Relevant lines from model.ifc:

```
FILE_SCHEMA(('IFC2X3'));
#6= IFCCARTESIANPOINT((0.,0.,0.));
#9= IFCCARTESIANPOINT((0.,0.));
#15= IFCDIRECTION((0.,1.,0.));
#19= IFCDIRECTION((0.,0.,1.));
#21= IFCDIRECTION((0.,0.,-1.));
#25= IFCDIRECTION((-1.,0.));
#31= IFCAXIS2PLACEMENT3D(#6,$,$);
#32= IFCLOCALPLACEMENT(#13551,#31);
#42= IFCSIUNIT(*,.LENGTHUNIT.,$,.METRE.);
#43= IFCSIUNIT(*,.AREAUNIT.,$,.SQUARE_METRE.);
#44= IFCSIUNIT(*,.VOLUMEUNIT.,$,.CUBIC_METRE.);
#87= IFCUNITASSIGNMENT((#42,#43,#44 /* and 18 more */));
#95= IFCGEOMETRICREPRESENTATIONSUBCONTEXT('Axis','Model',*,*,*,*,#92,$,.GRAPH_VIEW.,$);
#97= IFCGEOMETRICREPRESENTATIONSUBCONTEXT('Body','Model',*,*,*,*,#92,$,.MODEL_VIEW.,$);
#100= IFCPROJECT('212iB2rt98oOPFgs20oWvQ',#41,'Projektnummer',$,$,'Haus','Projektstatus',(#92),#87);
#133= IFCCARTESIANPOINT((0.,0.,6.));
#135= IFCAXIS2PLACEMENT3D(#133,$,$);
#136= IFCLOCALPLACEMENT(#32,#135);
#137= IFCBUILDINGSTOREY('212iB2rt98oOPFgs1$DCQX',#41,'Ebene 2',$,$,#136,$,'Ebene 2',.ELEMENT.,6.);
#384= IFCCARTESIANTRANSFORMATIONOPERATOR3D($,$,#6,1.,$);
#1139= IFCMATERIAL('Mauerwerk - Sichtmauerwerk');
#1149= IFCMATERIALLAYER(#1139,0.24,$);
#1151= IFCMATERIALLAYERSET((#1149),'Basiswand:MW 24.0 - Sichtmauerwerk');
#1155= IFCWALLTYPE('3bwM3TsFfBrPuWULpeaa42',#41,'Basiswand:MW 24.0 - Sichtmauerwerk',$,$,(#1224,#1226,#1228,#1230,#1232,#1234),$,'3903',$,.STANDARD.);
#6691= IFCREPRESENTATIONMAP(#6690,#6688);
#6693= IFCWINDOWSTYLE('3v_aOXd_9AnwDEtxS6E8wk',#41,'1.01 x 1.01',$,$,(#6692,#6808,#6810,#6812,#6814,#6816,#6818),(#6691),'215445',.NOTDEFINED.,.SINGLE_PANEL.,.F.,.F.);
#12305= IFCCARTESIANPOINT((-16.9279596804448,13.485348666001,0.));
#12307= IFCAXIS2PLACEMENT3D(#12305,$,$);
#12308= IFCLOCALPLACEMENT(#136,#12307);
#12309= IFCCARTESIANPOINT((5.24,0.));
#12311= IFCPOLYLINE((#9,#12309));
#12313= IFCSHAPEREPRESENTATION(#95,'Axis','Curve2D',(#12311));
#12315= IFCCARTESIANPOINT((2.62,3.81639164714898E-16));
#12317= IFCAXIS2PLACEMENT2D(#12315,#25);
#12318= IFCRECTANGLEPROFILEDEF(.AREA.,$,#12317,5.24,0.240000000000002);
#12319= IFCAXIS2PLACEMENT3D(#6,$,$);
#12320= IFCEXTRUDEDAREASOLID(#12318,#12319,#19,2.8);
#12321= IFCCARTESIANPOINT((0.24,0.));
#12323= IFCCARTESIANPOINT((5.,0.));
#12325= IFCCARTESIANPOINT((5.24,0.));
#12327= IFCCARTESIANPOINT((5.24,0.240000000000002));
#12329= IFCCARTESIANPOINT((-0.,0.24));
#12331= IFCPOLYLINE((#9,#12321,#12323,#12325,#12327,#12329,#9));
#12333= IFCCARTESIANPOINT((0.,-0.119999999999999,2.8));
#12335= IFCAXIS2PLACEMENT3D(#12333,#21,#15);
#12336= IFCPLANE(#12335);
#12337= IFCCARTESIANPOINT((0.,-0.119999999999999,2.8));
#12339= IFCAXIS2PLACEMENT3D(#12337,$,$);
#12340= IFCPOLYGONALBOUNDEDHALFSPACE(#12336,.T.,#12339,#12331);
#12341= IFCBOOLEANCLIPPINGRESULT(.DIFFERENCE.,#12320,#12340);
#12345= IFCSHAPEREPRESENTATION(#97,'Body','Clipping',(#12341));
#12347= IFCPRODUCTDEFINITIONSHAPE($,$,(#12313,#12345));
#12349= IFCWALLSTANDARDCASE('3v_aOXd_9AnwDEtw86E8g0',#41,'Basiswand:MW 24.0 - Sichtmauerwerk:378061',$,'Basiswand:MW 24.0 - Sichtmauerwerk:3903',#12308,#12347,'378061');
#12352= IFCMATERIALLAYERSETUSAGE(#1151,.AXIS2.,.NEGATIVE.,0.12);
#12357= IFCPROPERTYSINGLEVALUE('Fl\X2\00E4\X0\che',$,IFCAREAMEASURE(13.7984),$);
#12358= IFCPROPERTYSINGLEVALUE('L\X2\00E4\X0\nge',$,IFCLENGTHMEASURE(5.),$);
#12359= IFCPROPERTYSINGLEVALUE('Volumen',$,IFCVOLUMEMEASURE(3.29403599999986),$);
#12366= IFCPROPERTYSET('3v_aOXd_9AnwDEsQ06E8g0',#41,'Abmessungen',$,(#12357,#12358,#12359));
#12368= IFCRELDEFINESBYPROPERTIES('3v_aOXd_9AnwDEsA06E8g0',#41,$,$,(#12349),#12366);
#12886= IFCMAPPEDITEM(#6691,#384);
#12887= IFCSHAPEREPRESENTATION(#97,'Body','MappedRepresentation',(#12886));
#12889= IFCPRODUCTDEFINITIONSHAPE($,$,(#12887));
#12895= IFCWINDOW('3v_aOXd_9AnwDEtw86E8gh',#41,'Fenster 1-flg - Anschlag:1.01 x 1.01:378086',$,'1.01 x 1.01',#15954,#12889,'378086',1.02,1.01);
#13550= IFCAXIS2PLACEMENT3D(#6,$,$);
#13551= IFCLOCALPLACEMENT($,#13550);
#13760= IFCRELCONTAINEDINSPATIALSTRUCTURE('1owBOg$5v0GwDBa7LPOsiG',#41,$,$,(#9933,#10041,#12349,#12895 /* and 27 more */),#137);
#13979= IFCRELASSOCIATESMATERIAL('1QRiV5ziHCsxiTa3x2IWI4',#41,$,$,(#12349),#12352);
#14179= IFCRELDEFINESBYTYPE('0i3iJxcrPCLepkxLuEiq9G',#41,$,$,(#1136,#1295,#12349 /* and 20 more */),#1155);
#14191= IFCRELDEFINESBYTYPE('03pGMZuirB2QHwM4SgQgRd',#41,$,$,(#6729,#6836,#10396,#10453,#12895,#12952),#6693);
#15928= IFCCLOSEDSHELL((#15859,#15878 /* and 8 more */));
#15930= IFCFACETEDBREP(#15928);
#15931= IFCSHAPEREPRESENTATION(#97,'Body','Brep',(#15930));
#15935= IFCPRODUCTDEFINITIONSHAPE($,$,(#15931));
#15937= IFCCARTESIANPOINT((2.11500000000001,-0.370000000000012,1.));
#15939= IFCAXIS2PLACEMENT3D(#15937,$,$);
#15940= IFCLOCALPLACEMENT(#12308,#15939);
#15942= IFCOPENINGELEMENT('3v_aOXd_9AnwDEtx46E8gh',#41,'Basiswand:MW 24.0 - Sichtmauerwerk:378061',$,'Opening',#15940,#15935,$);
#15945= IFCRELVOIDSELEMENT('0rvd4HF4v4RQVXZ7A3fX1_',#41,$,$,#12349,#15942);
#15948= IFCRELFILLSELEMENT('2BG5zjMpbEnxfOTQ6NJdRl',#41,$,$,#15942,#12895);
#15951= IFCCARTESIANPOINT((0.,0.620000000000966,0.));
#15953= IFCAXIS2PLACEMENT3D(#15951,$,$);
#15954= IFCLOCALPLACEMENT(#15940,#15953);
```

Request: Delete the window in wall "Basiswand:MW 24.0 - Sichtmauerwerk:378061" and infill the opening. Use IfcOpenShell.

```python
import ifcopenshell
import ifcopenshell.api.feature
import ifcopenshell.api.pset
import ifcopenshell.api.root
import ifcopenshell.geom
import ifcopenshell.util.element
import ifcopenshell.util.shape
import ifcopenshell.util.unit

model = ifcopenshell.open("model.ifc")
area_scale = ifcopenshell.util.unit.calculate_unit_scale(model, "AREAUNIT")
volume_scale = ifcopenshell.util.unit.calculate_unit_scale(model, "VOLUMEUNIT")
settings = ifcopenshell.geom.settings()


def volume(element):
    """Net volume in cubic metres, openings subtracted."""
    shape = ifcopenshell.geom.create_shape(settings, element)
    return ifcopenshell.util.shape.get_volume(shape.geometry)


window = model.by_guid("3v_aOXd_9AnwDEtw86E8gh")
opening = window.FillsVoids[0].RelatingOpeningElement
wall = opening.VoidsElements[0].RelatingBuildingElement
before = volume(wall)

ifcopenshell.api.root.remove_product(model, product=window)
ifcopenshell.api.feature.remove_feature(model, feature=opening)

after = volume(wall)
thickness = 0.24  # wall thickness in metres

# Update the wall's stored quantities.
pset = model.by_id(ifcopenshell.util.element.get_pset(wall, "Abmessungen", should_inherit=False)["id"])
ifcopenshell.api.pset.edit_pset(model, pset=pset, properties={
    "Fläche": model.create_entity("IfcAreaMeasure", after / thickness / area_scale),
    "Volumen": model.create_entity("IfcVolumeMeasure", after / volume_scale),
})

print(f"wall volume {before:.3f} -> {after:.3f} m3")

model.write("model_v2.ifc")
```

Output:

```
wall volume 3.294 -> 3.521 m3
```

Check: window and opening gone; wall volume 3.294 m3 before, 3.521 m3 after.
